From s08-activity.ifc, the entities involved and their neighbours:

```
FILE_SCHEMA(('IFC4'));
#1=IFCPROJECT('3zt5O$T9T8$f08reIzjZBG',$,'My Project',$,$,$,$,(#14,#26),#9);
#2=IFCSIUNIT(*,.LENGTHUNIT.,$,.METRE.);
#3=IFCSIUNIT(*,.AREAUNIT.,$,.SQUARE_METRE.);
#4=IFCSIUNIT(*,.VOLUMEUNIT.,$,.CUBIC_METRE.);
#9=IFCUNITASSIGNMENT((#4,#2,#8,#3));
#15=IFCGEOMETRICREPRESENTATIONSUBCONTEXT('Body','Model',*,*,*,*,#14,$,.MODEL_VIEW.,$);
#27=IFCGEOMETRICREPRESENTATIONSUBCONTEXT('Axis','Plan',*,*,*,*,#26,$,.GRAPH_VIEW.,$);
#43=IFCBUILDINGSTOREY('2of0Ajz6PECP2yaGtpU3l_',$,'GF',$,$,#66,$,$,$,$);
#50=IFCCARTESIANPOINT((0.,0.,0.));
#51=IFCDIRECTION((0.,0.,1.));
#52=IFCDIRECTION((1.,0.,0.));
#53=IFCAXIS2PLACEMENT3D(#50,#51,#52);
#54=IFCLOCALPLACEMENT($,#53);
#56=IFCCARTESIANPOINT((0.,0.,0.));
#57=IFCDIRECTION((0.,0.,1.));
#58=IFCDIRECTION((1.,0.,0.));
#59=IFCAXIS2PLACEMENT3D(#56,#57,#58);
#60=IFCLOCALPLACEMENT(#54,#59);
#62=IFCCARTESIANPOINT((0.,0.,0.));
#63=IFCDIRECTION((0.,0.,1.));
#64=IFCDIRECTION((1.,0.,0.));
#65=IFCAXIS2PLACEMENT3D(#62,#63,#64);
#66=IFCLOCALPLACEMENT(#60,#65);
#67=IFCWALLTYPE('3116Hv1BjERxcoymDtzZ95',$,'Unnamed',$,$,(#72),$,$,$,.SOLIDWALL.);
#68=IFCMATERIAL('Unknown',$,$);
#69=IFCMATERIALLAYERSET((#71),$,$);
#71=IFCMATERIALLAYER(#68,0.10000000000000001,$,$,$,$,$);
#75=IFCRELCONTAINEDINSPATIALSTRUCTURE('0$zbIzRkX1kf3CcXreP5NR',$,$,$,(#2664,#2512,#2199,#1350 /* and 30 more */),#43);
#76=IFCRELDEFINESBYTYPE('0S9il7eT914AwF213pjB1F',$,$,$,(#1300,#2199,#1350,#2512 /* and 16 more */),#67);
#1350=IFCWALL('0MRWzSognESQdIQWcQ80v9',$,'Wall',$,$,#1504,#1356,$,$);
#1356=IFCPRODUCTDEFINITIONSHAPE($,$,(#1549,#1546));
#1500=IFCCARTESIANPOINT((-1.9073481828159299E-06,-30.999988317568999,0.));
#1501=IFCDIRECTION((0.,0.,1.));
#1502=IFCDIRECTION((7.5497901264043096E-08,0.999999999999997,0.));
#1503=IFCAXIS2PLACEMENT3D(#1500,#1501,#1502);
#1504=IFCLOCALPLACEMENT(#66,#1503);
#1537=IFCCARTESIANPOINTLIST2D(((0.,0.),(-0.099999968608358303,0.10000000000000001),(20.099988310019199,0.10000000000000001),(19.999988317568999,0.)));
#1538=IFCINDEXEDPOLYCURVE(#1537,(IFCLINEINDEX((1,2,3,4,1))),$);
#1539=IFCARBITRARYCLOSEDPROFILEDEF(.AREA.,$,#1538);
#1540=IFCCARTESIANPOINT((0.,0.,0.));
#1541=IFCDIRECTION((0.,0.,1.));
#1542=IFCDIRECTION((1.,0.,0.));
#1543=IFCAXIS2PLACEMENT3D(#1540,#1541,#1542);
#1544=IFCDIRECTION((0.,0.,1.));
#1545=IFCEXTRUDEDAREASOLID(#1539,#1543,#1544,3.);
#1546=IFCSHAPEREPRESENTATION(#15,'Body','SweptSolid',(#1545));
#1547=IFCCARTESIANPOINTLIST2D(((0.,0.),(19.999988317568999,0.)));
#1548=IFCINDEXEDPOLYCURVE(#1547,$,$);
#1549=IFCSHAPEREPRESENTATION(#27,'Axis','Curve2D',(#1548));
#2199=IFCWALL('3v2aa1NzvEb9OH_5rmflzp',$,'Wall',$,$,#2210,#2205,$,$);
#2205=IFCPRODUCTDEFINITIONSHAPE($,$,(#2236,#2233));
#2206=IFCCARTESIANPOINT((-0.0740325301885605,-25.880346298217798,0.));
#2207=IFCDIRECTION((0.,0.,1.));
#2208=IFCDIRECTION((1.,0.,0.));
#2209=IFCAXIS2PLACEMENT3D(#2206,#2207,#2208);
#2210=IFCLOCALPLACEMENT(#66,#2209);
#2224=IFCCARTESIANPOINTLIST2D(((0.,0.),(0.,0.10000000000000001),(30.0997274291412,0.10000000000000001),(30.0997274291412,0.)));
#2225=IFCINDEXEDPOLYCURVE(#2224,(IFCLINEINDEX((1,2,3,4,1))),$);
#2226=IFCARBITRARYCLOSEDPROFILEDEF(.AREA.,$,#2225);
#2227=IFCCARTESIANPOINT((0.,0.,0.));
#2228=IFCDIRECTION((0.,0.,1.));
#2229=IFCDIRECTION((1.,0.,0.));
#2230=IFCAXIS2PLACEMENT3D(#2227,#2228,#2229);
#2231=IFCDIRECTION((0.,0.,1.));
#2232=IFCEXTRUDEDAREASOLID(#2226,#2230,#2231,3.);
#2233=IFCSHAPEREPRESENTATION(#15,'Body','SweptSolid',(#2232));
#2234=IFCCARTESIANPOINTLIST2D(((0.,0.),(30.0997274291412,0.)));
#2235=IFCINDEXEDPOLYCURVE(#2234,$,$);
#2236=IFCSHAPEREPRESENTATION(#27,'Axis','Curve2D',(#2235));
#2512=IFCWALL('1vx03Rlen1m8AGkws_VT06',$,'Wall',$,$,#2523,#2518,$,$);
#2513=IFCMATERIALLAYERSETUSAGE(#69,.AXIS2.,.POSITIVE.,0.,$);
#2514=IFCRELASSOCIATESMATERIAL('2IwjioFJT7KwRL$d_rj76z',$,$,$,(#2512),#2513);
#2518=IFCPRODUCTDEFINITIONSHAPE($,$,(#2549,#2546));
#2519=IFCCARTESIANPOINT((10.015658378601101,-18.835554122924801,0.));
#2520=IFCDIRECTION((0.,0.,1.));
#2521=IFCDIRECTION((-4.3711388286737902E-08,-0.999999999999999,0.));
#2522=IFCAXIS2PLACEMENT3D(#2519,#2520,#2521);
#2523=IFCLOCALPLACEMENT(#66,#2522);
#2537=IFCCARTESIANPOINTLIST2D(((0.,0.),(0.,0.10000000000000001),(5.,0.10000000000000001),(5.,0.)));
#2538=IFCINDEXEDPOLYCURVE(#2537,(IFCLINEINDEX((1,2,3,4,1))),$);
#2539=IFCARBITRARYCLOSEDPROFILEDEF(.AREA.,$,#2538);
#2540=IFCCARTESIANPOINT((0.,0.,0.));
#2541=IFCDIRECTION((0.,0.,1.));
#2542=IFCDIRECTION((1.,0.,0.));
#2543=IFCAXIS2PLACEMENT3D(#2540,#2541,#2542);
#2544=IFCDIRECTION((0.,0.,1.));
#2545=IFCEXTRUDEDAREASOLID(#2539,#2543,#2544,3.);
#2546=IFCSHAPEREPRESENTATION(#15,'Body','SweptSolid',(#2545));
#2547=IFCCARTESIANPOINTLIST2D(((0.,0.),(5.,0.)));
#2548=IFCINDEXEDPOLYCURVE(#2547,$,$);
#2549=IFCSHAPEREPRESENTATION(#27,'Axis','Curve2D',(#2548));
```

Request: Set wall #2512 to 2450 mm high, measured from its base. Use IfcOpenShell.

```python
import ifcopenshell
import ifcopenshell.geom
import ifcopenshell.util.representation
import ifcopenshell.util.shape

model = ifcopenshell.open("s08-activity.ifc")
settings = ifcopenshell.geom.settings()


def volume(element):
    """Net volume in cubic metres, openings subtracted."""
    shape = ifcopenshell.geom.create_shape(settings, element)
    return ifcopenshell.util.shape.get_volume(shape.geometry)


wall = model.by_guid("1vx03Rlen1m8AGkws_VT06")
before = volume(wall)

body = ifcopenshell.util.representation.get_representation(wall, "Model", "Body")
solid = body.Items[0]
old_height = solid.Depth
solid.Depth = 2.45
after = volume(wall)

print(f"height {old_height:g} -> {solid.Depth:g}, volume {before:.3f} -> {after:.3f} m3")

model.write("s08-activity-out.ifc")
```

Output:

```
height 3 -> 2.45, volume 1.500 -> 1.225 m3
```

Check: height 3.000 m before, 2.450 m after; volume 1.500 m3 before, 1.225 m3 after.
